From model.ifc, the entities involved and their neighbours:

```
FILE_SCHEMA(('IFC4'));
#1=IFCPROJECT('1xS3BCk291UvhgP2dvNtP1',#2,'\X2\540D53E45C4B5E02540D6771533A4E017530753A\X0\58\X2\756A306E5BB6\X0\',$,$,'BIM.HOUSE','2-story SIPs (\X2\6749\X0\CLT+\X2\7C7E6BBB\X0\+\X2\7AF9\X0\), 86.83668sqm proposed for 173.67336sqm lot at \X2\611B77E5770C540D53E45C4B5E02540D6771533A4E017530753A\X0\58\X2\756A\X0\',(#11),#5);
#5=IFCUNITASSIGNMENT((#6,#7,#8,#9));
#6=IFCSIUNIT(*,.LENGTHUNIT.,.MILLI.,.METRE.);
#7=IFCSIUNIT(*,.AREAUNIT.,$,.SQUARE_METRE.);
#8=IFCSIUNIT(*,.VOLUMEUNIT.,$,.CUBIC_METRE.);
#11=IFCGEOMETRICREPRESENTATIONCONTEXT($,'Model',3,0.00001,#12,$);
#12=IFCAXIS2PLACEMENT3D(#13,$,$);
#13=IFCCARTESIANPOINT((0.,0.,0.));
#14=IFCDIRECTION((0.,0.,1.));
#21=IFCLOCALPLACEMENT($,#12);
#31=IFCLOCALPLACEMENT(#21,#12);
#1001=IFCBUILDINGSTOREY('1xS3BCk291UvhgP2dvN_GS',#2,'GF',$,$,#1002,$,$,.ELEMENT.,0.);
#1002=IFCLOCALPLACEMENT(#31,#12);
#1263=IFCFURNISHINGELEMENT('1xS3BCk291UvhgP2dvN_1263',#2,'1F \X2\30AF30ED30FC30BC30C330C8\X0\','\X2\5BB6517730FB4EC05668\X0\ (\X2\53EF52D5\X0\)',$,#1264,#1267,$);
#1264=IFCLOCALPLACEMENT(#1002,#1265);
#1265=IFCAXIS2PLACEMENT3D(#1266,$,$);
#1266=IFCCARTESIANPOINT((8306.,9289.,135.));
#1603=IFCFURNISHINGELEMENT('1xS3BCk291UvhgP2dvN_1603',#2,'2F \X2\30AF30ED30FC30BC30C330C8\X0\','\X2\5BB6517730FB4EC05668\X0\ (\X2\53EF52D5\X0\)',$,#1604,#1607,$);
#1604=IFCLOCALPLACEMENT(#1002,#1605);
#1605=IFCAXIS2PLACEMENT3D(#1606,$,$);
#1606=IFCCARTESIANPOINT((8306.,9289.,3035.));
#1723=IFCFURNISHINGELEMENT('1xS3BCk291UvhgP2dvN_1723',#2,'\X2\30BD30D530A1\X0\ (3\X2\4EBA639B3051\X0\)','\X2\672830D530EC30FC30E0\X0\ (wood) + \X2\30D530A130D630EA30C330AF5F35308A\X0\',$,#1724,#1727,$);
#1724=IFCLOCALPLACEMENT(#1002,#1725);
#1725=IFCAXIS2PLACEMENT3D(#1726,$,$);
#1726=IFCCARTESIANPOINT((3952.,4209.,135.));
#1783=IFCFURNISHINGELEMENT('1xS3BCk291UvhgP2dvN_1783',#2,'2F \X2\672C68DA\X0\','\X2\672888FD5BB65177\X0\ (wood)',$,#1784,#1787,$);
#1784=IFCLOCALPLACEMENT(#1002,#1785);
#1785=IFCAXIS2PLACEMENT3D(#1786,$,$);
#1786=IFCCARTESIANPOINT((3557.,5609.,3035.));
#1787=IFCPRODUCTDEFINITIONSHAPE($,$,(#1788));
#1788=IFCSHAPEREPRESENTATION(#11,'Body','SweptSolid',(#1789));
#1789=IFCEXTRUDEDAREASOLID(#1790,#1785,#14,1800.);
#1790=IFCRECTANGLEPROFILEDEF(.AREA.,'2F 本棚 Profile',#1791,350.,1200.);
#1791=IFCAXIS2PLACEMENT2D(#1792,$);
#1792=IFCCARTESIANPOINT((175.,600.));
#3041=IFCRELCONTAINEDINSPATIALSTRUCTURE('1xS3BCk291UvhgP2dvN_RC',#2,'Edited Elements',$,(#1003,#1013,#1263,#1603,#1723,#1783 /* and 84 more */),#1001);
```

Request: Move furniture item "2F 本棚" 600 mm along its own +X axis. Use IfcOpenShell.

```python
import ifcopenshell
import ifcopenshell.api.geometry
import ifcopenshell.util.placement

model = ifcopenshell.open("model.ifc")

item = model.by_id(1783)
matrix = ifcopenshell.util.placement.get_local_placement(item.ObjectPlacement)
matrix[:3, 3] += matrix[:3, 0] * 600.0
ifcopenshell.api.geometry.edit_object_placement(model, product=item, matrix=matrix, is_si=False)

print(ifcopenshell.util.placement.get_local_placement(item.ObjectPlacement).round(3) + 0.0)

model.write("model_edited.ifc")
```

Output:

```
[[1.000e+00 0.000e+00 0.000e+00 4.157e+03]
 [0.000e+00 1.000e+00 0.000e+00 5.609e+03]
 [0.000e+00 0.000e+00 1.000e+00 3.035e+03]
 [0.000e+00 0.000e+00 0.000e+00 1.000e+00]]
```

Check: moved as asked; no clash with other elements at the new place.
